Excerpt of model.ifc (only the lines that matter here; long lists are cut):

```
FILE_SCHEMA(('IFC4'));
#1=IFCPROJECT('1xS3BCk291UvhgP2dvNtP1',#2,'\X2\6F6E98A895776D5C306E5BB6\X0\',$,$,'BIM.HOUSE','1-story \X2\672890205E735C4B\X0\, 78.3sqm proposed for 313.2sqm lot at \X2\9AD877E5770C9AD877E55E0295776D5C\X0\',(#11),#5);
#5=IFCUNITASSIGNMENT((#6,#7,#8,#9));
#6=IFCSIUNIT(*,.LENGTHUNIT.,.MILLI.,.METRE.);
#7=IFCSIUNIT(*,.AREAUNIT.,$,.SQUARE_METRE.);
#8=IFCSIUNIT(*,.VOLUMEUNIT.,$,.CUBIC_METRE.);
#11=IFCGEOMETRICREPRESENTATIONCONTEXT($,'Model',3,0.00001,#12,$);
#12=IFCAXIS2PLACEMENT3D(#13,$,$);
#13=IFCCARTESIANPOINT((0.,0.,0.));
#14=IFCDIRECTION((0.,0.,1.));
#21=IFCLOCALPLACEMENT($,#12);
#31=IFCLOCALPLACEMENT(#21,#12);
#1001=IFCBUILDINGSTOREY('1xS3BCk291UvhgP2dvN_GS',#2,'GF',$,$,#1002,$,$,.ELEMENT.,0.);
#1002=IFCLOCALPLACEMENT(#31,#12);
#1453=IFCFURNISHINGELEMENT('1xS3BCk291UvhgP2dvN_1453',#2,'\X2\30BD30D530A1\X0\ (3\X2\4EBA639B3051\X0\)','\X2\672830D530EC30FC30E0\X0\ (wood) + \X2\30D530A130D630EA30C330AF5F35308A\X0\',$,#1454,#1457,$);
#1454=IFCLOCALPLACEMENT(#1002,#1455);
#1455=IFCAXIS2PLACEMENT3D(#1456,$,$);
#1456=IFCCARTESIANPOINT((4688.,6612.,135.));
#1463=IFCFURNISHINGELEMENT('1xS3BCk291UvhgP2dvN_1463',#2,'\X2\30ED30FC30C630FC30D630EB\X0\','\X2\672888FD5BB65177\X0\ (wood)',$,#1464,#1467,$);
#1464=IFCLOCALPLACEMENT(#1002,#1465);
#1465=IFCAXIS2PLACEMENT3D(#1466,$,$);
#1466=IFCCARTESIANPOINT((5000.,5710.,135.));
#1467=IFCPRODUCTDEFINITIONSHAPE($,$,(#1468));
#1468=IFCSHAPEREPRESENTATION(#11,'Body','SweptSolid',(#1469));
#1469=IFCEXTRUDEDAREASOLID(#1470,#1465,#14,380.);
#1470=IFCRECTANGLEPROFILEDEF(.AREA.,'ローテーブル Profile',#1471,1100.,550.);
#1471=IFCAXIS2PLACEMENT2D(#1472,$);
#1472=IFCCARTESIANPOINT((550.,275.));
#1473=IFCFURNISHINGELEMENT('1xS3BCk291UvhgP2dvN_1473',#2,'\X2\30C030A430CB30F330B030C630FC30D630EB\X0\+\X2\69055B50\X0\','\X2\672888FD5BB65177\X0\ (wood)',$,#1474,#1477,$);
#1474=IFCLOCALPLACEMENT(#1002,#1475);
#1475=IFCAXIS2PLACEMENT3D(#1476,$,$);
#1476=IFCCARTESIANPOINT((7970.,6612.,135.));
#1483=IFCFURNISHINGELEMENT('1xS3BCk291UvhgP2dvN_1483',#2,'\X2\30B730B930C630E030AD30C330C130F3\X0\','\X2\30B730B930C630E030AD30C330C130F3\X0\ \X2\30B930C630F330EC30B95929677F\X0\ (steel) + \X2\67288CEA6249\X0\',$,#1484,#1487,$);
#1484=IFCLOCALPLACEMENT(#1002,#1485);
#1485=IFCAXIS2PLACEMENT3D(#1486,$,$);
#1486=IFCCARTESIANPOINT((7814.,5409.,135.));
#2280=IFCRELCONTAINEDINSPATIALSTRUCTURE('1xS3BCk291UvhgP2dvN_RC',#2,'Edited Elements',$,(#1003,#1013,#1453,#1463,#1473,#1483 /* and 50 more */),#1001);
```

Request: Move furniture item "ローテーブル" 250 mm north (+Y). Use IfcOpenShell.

```python
import ifcopenshell
import ifcopenshell.api.geometry
import ifcopenshell.util.placement

model = ifcopenshell.open("model.ifc")

item = model.by_id(1463)
matrix = ifcopenshell.util.placement.get_local_placement(item.ObjectPlacement)
matrix[1, 3] += 250.0
ifcopenshell.api.geometry.edit_object_placement(model, product=item, matrix=matrix, is_si=False)

print(ifcopenshell.util.placement.get_local_placement(item.ObjectPlacement).round(3) + 0.0)

model.write("model_v2.ifc")
```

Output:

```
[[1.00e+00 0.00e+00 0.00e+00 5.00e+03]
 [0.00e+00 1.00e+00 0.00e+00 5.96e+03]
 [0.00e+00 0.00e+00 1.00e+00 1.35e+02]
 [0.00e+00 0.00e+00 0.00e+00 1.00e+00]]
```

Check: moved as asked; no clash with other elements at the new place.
